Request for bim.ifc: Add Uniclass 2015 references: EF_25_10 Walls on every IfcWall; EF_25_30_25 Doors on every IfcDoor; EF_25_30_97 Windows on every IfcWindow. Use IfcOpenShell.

First a look at what the model holds.

```python
import ifcopenshell

model = ifcopenshell.open("bim.ifc")
print(model.schema)
print("classifications:", [c.Name for c in model.by_type("IfcClassification")])
for ifc_class in ("IfcDoor", "IfcRoof", "IfcStair", "IfcWall", "IfcWindow"):
    print(ifc_class, len(model.by_type(ifc_class)))
```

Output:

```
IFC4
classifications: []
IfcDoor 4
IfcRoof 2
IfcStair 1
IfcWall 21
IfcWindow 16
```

```python
import ifcopenshell
import ifcopenshell.api.classification

model = ifcopenshell.open("bim.ifc")

system = ifcopenshell.api.classification.add_classification(model, classification="Uniclass 2015")

codes = {
    "IfcWall": ("EF_25_10", "Walls"),
    "IfcDoor": ("EF_25_30_25", "Doors"),
    "IfcWindow": ("EF_25_30_97", "Windows"),
}
for ifc_class, (code, name) in codes.items():
    products = model.by_type(ifc_class)
    ifcopenshell.api.classification.add_reference(
        model, products=products, classification=system, identification=code, name=name
    )
    print(code, len(products))

model.write("bim_rev.ifc")
```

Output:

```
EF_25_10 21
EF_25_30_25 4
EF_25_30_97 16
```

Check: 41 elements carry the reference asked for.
